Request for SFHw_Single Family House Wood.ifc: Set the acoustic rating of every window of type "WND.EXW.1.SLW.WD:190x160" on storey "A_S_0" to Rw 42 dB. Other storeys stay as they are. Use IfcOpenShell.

First a look at what the model holds.

```python
import ifcopenshell
import ifcopenshell.util.element

model = ifcopenshell.open("SFHw_Single Family House Wood.ifc")
print(model.schema)
storey = next(s for s in model.by_type("IfcBuildingStorey") if s.Name == "A_S_0")
windows = [e for e in ifcopenshell.util.element.get_decomposition(storey) if e.is_a("IfcWindow")]
seen = {}
for e in windows:
    element_type = ifcopenshell.util.element.get_type(e)
    key = (element_type.Name if element_type != e and element_type else None, ifcopenshell.util.element.get_pset(e, "Pset_WindowCommon", "AcousticRating"))
    seen[key] = seen.get(key, 0) + 1
for (name, value), count in sorted(seen.items(), key=str):
    print(count, "x", name, "|", value)
```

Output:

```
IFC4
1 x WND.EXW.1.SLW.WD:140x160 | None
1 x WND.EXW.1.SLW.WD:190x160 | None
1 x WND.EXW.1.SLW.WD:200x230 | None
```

```python
import ifcopenshell
import ifcopenshell.api.pset
import ifcopenshell.util.element

model = ifcopenshell.open("SFHw_Single Family House Wood.ifc")

storey = next(s for s in model.by_type("IfcBuildingStorey") if s.Name == "A_S_0")
windows = [e for e in ifcopenshell.util.element.get_decomposition(storey) if e.is_a("IfcWindow")]

count = 0
for e in windows:
    element_type = ifcopenshell.util.element.get_type(e)
    if element_type in (None, e) or element_type.Name != "WND.EXW.1.SLW.WD:190x160":
        continue
    # add_pset returns the element's existing set when there is one.
    pset = ifcopenshell.api.pset.add_pset(model, product=e, name="Pset_WindowCommon")
    ifcopenshell.api.pset.edit_pset(model, pset=pset, properties={"AcousticRating": "Rw 42 dB"})
    count += 1

print(count, "windows updated")

model.write("SFHw_Single Family House Wood_rev.ifc")
```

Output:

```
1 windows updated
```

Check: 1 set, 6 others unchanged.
